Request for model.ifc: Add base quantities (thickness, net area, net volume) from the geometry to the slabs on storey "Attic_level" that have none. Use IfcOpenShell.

First a look at what the model holds.

```python
import ifcopenshell
import ifcopenshell.util.element
import ifcopenshell.util.unit

model = ifcopenshell.open("model.ifc")
print(model.schema)
for unit_type in ("LENGTHUNIT", "AREAUNIT", "VOLUMEUNIT"):
    print(unit_type, ifcopenshell.util.unit.calculate_unit_scale(model, unit_type))
storey = next(s for s in model.by_type("IfcBuildingStorey") if s.Name == "Attic_level")
slabs = [e for e in ifcopenshell.util.element.get_decomposition(storey) if e.is_a("IfcSlab")]
for e in sorted(slabs, key=lambda e: e.id()):
    print(e.id(), e.is_a(), e.Name, list(ifcopenshell.util.element.get_psets(e, qtos_only=True)), sep=" | ")
```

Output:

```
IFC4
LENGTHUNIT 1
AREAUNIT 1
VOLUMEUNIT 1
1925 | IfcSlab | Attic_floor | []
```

```python
import ifcopenshell
import ifcopenshell.api.pset
import ifcopenshell.geom
import ifcopenshell.util.element
import ifcopenshell.util.shape
import ifcopenshell.util.unit

model = ifcopenshell.open("model.ifc")
unit_scale = ifcopenshell.util.unit.calculate_unit_scale(model)
area_scale = ifcopenshell.util.unit.calculate_unit_scale(model, "AREAUNIT")
volume_scale = ifcopenshell.util.unit.calculate_unit_scale(model, "VOLUMEUNIT")
settings = ifcopenshell.geom.settings()

storey = next(s for s in model.by_type("IfcBuildingStorey") if s.Name == "Attic_level")
slabs = [e for e in ifcopenshell.util.element.get_decomposition(storey) if e.is_a("IfcSlab")]

for e in sorted(slabs, key=lambda e: e.id()):
    if ifcopenshell.util.element.get_psets(e, qtos_only=True, should_inherit=False):
        continue
    # Geometry comes back in metres, in the element's own axes.
    shape = ifcopenshell.geom.create_shape(settings, e)
    values = {
        "Width": ifcopenshell.util.shape.get_z(shape.geometry) / unit_scale,
        "NetArea": ifcopenshell.util.shape.get_footprint_area(shape.geometry) / area_scale,
        "NetVolume": ifcopenshell.util.shape.get_volume(shape.geometry) / volume_scale,
    }
    qto = ifcopenshell.api.pset.add_qto(model, product=e, name="Qto_SlabBaseQuantities")
    ifcopenshell.api.pset.edit_qto(model, qto=qto, properties=values)
    print(e.id(), {k: round(v, 3) for k, v in values.items()})

model.write("model_v2.ifc")
```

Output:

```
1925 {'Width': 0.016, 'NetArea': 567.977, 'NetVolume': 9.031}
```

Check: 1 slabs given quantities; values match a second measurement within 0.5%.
